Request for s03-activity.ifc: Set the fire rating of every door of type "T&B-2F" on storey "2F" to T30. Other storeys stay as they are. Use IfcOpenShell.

First a look at what the model holds.

```python
import ifcopenshell
import ifcopenshell.util.element

model = ifcopenshell.open("s03-activity.ifc")
print(model.schema)
storey = next(s for s in model.by_type("IfcBuildingStorey") if s.Name == "2F")
doors = [e for e in ifcopenshell.util.element.get_decomposition(storey) if e.is_a("IfcDoor")]
seen = {}
for e in doors:
    element_type = ifcopenshell.util.element.get_type(e)
    key = (element_type.Name if element_type != e and element_type else None, ifcopenshell.util.element.get_pset(e, "Pset_DoorCommon", "FireRating"))
    seen[key] = seen.get(key, 0) + 1
for (name, value), count in sorted(seen.items(), key=str):
    print(count, "x", name, "|", value)
```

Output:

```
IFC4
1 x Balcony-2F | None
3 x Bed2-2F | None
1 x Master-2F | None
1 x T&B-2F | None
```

```python
import ifcopenshell
import ifcopenshell.api.pset
import ifcopenshell.util.element

model = ifcopenshell.open("s03-activity.ifc")

storey = next(s for s in model.by_type("IfcBuildingStorey") if s.Name == "2F")
doors = [e for e in ifcopenshell.util.element.get_decomposition(storey) if e.is_a("IfcDoor")]

count = 0
for e in doors:
    element_type = ifcopenshell.util.element.get_type(e)
    if element_type in (None, e) or element_type.Name != "T&B-2F":
        continue
    # add_pset returns the element's existing set when there is one.
    pset = ifcopenshell.api.pset.add_pset(model, product=e, name="Pset_DoorCommon")
    ifcopenshell.api.pset.edit_pset(model, pset=pset, properties={"FireRating": "T30"})
    count += 1

print(count, "doors updated")

model.write("s03-activity_edited.ifc")
```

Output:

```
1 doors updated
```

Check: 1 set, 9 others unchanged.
